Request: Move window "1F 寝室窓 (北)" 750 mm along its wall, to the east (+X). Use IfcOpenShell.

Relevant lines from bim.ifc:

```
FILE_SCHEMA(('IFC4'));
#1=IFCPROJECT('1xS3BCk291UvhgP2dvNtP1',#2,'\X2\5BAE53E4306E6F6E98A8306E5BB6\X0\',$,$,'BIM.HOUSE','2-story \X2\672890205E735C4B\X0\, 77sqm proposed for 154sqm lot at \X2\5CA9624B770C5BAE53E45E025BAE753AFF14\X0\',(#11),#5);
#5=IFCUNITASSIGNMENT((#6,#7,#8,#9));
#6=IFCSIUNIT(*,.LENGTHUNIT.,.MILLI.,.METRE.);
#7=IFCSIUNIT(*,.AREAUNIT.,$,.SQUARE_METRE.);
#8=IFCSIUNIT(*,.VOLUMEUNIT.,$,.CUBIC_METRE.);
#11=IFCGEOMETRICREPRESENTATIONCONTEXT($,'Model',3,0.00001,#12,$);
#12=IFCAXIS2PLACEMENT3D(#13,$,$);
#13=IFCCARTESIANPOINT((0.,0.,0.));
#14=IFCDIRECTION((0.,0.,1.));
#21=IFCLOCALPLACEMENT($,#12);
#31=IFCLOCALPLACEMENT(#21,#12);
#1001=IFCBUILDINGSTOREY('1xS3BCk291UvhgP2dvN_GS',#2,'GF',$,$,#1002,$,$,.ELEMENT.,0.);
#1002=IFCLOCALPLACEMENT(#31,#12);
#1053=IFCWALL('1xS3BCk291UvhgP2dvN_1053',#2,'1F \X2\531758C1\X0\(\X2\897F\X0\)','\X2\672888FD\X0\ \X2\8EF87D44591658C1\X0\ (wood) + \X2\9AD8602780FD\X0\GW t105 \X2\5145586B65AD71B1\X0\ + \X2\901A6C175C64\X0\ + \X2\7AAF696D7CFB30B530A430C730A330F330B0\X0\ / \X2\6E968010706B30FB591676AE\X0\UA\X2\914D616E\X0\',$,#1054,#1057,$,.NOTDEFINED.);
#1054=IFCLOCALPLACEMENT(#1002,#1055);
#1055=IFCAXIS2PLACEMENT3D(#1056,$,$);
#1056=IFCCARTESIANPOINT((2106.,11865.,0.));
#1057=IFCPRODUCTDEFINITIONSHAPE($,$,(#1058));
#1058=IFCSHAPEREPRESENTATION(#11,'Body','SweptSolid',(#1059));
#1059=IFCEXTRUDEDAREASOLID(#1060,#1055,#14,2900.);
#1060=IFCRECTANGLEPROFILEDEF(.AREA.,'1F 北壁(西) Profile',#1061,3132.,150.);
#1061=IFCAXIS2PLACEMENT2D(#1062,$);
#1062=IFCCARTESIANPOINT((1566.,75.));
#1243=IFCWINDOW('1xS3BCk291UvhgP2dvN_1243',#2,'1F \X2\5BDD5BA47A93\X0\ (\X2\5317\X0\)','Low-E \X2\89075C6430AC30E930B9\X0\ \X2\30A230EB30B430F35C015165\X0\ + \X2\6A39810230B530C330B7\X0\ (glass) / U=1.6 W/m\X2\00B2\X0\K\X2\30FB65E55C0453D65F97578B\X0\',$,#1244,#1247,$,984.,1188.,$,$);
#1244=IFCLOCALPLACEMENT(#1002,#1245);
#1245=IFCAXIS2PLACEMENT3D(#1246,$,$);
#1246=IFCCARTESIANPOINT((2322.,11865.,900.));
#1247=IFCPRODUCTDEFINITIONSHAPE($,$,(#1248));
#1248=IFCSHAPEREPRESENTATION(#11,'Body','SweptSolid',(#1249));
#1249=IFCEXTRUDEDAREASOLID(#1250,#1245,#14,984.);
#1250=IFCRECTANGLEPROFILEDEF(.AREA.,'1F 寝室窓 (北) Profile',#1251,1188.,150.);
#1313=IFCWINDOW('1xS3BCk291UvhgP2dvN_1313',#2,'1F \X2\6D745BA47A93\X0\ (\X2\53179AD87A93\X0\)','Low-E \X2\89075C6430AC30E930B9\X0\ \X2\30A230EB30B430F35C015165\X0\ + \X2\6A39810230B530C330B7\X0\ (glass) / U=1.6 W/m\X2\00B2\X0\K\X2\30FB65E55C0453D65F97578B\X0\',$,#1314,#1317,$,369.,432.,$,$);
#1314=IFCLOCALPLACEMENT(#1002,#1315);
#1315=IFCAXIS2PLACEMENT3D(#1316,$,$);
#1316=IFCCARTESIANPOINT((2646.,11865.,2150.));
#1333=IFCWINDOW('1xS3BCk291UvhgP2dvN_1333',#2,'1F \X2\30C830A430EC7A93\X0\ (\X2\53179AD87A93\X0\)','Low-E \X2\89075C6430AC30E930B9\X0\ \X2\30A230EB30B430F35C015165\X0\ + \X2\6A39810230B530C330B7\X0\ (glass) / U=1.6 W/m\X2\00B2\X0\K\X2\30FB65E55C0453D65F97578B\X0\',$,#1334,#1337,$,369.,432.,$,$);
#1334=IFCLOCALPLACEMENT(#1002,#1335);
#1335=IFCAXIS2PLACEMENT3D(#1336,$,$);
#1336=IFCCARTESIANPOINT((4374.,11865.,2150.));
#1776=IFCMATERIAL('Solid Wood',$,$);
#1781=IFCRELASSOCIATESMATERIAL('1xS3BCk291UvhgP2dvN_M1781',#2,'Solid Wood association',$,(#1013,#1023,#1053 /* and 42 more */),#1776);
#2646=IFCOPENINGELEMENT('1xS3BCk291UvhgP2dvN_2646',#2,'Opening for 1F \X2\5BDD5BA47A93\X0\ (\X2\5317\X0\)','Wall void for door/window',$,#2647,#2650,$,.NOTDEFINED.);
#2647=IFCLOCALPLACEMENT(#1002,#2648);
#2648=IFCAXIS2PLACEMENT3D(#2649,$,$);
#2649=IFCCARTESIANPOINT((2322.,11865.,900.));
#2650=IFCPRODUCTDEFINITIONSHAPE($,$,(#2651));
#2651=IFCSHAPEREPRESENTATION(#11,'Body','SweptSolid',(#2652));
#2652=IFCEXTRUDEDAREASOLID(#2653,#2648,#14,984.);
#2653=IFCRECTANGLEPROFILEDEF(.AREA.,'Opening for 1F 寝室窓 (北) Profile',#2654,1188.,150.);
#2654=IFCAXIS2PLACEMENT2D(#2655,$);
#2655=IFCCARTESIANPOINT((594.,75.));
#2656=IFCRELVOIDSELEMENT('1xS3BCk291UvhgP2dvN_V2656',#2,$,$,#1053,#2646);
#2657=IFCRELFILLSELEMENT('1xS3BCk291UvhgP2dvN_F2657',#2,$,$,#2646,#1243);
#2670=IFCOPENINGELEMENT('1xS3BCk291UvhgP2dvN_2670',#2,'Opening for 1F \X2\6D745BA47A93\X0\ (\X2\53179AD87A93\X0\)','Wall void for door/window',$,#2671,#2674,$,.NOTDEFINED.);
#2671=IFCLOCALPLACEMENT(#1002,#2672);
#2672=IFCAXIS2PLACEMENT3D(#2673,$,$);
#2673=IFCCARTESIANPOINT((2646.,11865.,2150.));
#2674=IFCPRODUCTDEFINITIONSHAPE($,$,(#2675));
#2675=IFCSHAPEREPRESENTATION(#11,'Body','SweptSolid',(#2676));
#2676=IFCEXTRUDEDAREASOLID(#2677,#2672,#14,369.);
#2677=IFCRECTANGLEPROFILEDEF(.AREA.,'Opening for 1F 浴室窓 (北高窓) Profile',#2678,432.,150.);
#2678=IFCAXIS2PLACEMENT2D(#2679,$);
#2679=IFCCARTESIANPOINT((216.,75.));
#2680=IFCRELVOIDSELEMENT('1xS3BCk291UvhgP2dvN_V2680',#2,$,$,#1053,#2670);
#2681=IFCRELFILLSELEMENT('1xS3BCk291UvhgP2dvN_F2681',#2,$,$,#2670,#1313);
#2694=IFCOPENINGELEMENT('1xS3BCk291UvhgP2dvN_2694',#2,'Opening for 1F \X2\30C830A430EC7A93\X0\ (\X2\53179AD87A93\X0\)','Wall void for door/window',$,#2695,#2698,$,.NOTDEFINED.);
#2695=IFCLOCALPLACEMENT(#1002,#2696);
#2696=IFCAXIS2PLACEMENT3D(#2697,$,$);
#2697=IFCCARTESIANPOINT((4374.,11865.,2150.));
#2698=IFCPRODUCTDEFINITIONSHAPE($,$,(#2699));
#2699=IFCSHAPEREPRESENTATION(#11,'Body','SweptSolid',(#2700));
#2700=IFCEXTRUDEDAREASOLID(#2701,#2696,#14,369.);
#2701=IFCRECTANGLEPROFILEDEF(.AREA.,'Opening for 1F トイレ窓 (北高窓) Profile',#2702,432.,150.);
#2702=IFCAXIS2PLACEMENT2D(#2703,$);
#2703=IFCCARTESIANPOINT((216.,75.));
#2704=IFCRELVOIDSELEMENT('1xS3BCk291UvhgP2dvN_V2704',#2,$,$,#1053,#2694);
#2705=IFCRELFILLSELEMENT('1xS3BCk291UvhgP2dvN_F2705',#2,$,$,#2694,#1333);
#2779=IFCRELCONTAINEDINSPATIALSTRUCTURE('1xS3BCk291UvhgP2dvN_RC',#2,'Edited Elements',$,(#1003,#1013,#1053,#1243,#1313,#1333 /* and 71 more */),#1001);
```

```python
import ifcopenshell
import ifcopenshell.api.geometry
import ifcopenshell.util.placement

model = ifcopenshell.open("bim.ifc")

window = model.by_guid("1xS3BCk291UvhgP2dvN_1243")
opening = window.FillsVoids[0].RelatingOpeningElement
wall = opening.VoidsElements[0].RelatingBuildingElement

wall_matrix = ifcopenshell.util.placement.get_local_placement(wall.ObjectPlacement)
shift = wall_matrix[:3, 0] * 750.0
before = ifcopenshell.util.placement.get_local_placement(window.ObjectPlacement)[:3, 3].copy()

# The window is not placed relative to its opening, so move both.
for product in (opening, window):
    matrix = ifcopenshell.util.placement.get_local_placement(product.ObjectPlacement)
    matrix[:3, 3] += shift
    ifcopenshell.api.geometry.edit_object_placement(model, product=product, matrix=matrix, is_si=False)

after = ifcopenshell.util.placement.get_local_placement(window.ObjectPlacement)[:3, 3]
print("window moved by", (after - before).round(3) + 0.0)

model.write("bim_v2.ifc")
```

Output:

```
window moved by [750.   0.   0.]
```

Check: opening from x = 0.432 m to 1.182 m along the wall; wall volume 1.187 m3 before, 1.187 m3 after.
